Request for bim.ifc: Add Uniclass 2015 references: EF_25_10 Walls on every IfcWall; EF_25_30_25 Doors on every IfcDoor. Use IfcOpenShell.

First a look at what the model holds.

```python
import ifcopenshell

model = ifcopenshell.open("bim.ifc")
print(model.schema)
print("classifications:", [c.Name for c in model.by_type("IfcClassification")])
for ifc_class in ("IfcDoor", "IfcRoof", "IfcStair", "IfcWall", "IfcWindow"):
    print(ifc_class, len(model.by_type(ifc_class)))
```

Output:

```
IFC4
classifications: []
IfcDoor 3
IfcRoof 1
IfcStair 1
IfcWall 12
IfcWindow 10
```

```python
import ifcopenshell
import ifcopenshell.api.classification

model = ifcopenshell.open("bim.ifc")

system = ifcopenshell.api.classification.add_classification(model, classification="Uniclass 2015")

codes = {
    "IfcWall": ("EF_25_10", "Walls"),
    "IfcDoor": ("EF_25_30_25", "Doors"),
}
for ifc_class, (code, name) in codes.items():
    products = model.by_type(ifc_class)
    ifcopenshell.api.classification.add_reference(
        model, products=products, classification=system, identification=code, name=name
    )
    print(code, len(products))

model.write("bim-out.ifc")
```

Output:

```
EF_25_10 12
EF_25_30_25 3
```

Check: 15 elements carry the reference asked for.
